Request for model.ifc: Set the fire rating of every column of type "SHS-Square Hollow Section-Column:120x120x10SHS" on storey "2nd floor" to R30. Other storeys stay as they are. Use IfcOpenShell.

First a look at what the model holds.

```python
import ifcopenshell
import ifcopenshell.util.element

model = ifcopenshell.open("model.ifc")
print(model.schema)
storey = next(s for s in model.by_type("IfcBuildingStorey") if s.Name == "2nd floor")
columns = [e for e in ifcopenshell.util.element.get_decomposition(storey) if e.is_a("IfcColumn")]
seen = {}
for e in columns:
    element_type = ifcopenshell.util.element.get_type(e)
    key = (element_type.Name if element_type != e and element_type else None, ifcopenshell.util.element.get_pset(e, "Pset_ColumnCommon", "FireRating"))
    seen[key] = seen.get(key, 0) + 1
for (name, value), count in sorted(seen.items(), key=str):
    print(count, "x", name, "|", value)
```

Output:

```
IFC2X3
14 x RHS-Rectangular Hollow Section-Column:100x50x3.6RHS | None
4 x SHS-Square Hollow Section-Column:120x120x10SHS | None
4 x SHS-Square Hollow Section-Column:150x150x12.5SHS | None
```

```python
import ifcopenshell
import ifcopenshell.api.pset
import ifcopenshell.util.element

model = ifcopenshell.open("model.ifc")

storey = next(s for s in model.by_type("IfcBuildingStorey") if s.Name == "2nd floor")
columns = [e for e in ifcopenshell.util.element.get_decomposition(storey) if e.is_a("IfcColumn")]

count = 0
for e in columns:
    element_type = ifcopenshell.util.element.get_type(e)
    if element_type in (None, e) or element_type.Name != "SHS-Square Hollow Section-Column:120x120x10SHS":
        continue
    # add_pset returns the element's existing set when there is one.
    pset = ifcopenshell.api.pset.add_pset(model, product=e, name="Pset_ColumnCommon")
    ifcopenshell.api.pset.edit_pset(model, pset=pset, properties={"FireRating": "R30"})
    count += 1

print(count, "columns updated")

model.write("model-out.ifc")
```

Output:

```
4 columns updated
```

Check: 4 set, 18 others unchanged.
